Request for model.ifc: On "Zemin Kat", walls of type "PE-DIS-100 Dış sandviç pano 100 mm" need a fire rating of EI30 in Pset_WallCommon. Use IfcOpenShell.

First a look at what the model holds.

```python
import ifcopenshell
import ifcopenshell.util.element

model = ifcopenshell.open("model.ifc")
print(model.schema)
storey = next(s for s in model.by_type("IfcBuildingStorey") if s.Name == "Zemin Kat")
walls = [e for e in ifcopenshell.util.element.get_decomposition(storey) if e.is_a("IfcWall")]
seen = {}
for e in walls:
    element_type = ifcopenshell.util.element.get_type(e)
    key = (element_type.Name if element_type != e and element_type else None, ifcopenshell.util.element.get_pset(e, "Pset_WallCommon", "FireRating"))
    seen[key] = seen.get(key, 0) + 1
for (name, value), count in sorted(seen.items(), key=str):
    print(count, "x", name, "|", value)
```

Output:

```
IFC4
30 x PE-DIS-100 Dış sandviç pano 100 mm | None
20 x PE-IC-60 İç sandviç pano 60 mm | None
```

```python
import ifcopenshell
import ifcopenshell.api.pset
import ifcopenshell.util.element

model = ifcopenshell.open("model.ifc")

storey = next(s for s in model.by_type("IfcBuildingStorey") if s.Name == "Zemin Kat")
walls = [e for e in ifcopenshell.util.element.get_decomposition(storey) if e.is_a("IfcWall")]

count = 0
for e in walls:
    element_type = ifcopenshell.util.element.get_type(e)
    if element_type in (None, e) or element_type.Name != "PE-DIS-100 Dış sandviç pano 100 mm":
        continue
    # add_pset returns the element's existing set when there is one.
    pset = ifcopenshell.api.pset.add_pset(model, product=e, name="Pset_WallCommon")
    ifcopenshell.api.pset.edit_pset(model, pset=pset, properties={"FireRating": "EI30"})
    count += 1

print(count, "walls updated")

model.write("model-out.ifc")
```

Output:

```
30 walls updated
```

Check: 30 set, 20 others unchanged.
